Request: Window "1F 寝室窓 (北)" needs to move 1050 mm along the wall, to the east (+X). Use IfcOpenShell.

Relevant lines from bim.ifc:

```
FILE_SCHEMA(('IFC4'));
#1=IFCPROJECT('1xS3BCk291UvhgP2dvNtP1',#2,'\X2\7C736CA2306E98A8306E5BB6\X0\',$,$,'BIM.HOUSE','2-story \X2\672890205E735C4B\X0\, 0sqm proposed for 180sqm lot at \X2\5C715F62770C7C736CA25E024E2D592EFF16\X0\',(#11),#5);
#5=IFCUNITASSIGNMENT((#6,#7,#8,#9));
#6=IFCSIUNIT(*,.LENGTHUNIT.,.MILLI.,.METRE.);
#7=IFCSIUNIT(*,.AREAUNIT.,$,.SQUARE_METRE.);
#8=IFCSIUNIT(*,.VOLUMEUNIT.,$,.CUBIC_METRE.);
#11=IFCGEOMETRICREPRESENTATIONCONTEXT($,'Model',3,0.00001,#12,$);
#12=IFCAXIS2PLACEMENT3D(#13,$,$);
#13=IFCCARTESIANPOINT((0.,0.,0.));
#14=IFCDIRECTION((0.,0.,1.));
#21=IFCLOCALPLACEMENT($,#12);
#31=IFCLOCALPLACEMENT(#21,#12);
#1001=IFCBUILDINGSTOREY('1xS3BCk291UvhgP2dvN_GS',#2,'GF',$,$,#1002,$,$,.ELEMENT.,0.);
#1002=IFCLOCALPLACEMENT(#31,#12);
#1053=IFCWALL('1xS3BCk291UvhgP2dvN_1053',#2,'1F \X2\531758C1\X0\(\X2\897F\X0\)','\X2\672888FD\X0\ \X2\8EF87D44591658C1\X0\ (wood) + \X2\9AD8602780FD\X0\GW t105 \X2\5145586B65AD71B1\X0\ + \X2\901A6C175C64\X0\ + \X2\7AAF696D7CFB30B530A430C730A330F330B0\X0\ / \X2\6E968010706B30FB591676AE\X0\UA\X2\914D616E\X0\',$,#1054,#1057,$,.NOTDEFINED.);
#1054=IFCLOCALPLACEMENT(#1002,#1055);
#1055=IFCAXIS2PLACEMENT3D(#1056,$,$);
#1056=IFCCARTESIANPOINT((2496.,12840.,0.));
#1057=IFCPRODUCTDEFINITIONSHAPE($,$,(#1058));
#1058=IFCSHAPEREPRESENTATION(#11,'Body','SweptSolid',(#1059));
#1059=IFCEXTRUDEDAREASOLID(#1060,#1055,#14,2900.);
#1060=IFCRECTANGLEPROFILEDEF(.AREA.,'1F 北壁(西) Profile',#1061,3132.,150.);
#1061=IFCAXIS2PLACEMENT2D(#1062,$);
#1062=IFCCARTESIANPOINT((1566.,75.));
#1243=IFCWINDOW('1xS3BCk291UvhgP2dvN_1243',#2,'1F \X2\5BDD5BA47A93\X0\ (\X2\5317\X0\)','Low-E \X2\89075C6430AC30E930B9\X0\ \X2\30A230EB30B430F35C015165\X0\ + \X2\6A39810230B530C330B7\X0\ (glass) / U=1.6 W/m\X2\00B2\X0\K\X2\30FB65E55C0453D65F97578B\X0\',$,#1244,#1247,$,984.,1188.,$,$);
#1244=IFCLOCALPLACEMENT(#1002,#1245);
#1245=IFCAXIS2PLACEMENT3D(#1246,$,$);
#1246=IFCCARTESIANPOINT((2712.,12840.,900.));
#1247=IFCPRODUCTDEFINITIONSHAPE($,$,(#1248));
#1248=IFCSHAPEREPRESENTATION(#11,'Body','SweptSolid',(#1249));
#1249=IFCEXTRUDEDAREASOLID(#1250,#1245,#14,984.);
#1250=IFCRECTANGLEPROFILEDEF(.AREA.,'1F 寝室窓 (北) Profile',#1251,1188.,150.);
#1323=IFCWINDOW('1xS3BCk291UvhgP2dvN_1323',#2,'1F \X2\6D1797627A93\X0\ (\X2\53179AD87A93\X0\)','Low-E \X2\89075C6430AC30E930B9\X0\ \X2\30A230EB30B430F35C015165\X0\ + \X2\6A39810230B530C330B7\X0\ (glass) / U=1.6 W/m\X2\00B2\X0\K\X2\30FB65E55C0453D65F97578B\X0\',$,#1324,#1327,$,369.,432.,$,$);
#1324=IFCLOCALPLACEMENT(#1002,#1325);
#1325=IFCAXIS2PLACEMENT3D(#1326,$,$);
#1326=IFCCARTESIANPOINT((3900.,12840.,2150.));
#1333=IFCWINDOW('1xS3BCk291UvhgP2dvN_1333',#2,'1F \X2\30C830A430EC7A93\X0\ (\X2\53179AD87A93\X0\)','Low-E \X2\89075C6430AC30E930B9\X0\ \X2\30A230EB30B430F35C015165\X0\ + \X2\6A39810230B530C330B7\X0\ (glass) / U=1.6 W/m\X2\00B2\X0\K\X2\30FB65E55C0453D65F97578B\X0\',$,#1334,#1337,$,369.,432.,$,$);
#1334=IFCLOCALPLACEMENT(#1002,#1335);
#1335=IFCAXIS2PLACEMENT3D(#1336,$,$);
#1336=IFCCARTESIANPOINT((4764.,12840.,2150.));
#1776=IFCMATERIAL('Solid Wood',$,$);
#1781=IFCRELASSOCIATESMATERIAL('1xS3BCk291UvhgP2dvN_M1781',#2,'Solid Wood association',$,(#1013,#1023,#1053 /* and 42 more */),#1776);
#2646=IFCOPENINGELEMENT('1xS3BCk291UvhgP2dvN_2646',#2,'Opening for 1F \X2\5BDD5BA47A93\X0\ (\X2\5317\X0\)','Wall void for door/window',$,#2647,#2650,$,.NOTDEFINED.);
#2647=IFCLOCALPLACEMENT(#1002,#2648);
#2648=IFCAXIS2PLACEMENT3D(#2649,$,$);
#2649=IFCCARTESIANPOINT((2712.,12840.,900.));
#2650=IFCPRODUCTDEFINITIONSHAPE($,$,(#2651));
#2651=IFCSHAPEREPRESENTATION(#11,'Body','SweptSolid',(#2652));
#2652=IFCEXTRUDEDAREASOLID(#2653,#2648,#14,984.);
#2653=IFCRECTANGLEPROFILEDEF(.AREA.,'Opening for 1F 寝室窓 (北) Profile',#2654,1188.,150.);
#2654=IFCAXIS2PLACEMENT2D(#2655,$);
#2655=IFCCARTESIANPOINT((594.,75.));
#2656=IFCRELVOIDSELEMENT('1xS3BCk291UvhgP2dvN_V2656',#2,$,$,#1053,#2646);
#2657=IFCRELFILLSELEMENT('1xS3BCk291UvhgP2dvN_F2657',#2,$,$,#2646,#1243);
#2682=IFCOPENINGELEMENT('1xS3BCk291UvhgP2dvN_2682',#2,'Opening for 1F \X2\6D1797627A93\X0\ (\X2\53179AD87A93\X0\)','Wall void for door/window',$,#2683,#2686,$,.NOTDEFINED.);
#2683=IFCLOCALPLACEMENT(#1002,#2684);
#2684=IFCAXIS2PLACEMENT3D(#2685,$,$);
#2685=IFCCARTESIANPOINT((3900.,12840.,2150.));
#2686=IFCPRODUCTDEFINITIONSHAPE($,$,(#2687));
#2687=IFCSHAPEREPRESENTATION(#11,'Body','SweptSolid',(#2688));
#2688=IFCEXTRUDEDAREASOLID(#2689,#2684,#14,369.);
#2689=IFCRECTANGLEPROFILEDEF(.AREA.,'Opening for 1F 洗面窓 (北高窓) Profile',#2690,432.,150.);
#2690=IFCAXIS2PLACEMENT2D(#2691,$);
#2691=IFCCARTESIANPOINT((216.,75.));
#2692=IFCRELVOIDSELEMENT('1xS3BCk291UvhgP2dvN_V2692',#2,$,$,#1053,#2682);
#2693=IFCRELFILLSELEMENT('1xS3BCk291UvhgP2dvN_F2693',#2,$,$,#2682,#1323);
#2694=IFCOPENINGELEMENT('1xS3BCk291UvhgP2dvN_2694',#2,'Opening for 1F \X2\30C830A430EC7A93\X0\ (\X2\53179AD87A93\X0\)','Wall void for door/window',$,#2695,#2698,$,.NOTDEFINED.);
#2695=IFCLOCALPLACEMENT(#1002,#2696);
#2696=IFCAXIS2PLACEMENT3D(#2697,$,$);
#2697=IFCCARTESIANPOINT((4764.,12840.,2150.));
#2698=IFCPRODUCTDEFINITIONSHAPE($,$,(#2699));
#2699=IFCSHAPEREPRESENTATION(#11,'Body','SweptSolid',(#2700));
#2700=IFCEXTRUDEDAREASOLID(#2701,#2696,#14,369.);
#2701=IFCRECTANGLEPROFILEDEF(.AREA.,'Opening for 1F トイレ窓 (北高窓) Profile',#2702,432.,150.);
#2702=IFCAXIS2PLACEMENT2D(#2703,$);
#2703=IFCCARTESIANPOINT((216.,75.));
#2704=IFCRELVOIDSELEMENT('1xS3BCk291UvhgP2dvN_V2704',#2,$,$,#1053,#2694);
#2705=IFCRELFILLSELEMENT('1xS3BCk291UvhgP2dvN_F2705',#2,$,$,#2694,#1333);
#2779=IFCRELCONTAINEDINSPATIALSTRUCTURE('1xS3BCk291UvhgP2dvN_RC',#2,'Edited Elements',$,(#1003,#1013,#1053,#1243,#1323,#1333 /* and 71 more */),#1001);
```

```python
import ifcopenshell
import ifcopenshell.api.geometry
import ifcopenshell.util.placement

model = ifcopenshell.open("bim.ifc")

window = model.by_guid("1xS3BCk291UvhgP2dvN_1243")
opening = window.FillsVoids[0].RelatingOpeningElement
wall = opening.VoidsElements[0].RelatingBuildingElement

wall_matrix = ifcopenshell.util.placement.get_local_placement(wall.ObjectPlacement)
shift = wall_matrix[:3, 0] * 1050.0
before = ifcopenshell.util.placement.get_local_placement(window.ObjectPlacement)[:3, 3].copy()

# The window is not placed relative to its opening, so move both.
for product in (opening, window):
    matrix = ifcopenshell.util.placement.get_local_placement(product.ObjectPlacement)
    matrix[:3, 3] += shift
    ifcopenshell.api.geometry.edit_object_placement(model, product=product, matrix=matrix, is_si=False)

after = ifcopenshell.util.placement.get_local_placement(window.ObjectPlacement)[:3, 3]
print("window moved by", (after - before).round(3) + 0.0)

model.write("bim_updated.ifc")
```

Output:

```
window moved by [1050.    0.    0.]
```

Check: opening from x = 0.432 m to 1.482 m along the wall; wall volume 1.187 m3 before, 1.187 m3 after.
